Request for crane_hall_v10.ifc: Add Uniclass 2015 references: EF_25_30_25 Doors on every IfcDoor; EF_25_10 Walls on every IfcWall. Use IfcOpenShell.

First a look at what the model holds.

```python
import ifcopenshell

model = ifcopenshell.open("crane_hall_v10.ifc")
print(model.schema)
print("classifications:", [c.Name for c in model.by_type("IfcClassification")])
for ifc_class in ("IfcDoor", "IfcRoof", "IfcStair", "IfcWall", "IfcWindow"):
    print(ifc_class, len(model.by_type(ifc_class)))
```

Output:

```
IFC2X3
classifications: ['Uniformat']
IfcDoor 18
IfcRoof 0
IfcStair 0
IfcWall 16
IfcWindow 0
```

```python
import ifcopenshell
import ifcopenshell.api.classification

model = ifcopenshell.open("crane_hall_v10.ifc")

# IFC2X3 requires Source and Edition and has no link from the project to the system.
system = model.create_entity("IfcClassification", Source="NBS", Edition="2015", Name="Uniclass 2015")

codes = {
    "IfcDoor": ("EF_25_30_25", "Doors"),
    "IfcWall": ("EF_25_10", "Walls"),
}
for ifc_class, (code, name) in codes.items():
    products = model.by_type(ifc_class)
    ifcopenshell.api.classification.add_reference(
        model, products=products, classification=system, identification=code, name=name
    )
    print(code, len(products))

model.write("crane_hall_v10_updated.ifc")
```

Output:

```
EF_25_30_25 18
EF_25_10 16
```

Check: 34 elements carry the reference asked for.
